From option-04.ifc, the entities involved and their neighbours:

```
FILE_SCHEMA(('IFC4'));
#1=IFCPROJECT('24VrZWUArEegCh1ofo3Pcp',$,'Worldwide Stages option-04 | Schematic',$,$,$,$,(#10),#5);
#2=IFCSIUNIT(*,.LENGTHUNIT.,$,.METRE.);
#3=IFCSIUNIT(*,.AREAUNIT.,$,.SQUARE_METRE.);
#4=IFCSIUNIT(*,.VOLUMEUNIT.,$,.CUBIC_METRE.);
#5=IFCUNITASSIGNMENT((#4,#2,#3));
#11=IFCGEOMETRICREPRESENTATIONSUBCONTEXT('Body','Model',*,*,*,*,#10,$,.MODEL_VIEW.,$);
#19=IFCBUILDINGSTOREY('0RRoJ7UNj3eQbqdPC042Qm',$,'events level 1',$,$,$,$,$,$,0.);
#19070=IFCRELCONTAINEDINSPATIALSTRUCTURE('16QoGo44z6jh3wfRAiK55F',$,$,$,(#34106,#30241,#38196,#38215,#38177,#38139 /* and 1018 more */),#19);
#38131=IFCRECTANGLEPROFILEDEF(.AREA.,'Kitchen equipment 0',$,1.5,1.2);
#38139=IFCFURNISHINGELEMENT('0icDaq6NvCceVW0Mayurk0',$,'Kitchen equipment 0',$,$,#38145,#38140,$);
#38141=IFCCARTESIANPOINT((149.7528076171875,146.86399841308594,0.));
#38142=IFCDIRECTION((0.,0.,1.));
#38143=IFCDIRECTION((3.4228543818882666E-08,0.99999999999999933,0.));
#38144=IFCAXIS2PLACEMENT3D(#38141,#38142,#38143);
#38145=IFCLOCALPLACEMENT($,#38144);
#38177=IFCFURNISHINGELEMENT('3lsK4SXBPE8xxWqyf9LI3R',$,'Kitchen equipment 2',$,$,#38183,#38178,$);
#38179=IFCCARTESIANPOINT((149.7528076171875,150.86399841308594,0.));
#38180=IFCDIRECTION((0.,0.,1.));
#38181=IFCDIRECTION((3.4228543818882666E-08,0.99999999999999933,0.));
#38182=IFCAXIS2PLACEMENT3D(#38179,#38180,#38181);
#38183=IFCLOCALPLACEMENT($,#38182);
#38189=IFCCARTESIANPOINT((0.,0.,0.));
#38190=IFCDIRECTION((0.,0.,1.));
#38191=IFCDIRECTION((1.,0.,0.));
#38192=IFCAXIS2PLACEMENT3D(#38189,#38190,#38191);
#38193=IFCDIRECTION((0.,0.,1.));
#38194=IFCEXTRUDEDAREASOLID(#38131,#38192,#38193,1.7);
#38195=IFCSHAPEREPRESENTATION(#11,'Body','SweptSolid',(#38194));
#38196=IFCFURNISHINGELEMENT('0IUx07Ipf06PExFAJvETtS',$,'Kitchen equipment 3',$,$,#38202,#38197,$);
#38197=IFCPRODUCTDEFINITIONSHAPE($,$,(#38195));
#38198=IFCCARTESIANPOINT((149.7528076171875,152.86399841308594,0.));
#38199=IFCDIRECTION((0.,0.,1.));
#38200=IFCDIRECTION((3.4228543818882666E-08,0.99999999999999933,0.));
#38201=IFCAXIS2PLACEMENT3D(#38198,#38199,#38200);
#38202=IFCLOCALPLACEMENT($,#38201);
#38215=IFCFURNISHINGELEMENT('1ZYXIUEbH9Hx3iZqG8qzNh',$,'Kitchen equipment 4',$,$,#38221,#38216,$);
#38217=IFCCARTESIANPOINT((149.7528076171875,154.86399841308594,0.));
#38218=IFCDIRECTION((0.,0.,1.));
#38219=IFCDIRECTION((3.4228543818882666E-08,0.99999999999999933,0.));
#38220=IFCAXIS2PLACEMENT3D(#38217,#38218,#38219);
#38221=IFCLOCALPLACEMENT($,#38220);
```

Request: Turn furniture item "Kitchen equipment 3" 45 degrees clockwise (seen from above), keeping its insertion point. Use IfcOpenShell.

```python
import ifcopenshell
import ifcopenshell.api.geometry
import ifcopenshell.util.placement

model = ifcopenshell.open("option-04.ifc")

item = model.by_id(38196)
matrix = ifcopenshell.util.placement.get_local_placement(item.ObjectPlacement)
matrix = matrix @ ifcopenshell.util.placement.rotation(-45, "Z")
ifcopenshell.api.geometry.edit_object_placement(model, product=item, matrix=matrix, is_si=False)

print(ifcopenshell.util.placement.get_local_placement(item.ObjectPlacement).round(3) + 0.0)

model.write("option-04_updated.ifc")
```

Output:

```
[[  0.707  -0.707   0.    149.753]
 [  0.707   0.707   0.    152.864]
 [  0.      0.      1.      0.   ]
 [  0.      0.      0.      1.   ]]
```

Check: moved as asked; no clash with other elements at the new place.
